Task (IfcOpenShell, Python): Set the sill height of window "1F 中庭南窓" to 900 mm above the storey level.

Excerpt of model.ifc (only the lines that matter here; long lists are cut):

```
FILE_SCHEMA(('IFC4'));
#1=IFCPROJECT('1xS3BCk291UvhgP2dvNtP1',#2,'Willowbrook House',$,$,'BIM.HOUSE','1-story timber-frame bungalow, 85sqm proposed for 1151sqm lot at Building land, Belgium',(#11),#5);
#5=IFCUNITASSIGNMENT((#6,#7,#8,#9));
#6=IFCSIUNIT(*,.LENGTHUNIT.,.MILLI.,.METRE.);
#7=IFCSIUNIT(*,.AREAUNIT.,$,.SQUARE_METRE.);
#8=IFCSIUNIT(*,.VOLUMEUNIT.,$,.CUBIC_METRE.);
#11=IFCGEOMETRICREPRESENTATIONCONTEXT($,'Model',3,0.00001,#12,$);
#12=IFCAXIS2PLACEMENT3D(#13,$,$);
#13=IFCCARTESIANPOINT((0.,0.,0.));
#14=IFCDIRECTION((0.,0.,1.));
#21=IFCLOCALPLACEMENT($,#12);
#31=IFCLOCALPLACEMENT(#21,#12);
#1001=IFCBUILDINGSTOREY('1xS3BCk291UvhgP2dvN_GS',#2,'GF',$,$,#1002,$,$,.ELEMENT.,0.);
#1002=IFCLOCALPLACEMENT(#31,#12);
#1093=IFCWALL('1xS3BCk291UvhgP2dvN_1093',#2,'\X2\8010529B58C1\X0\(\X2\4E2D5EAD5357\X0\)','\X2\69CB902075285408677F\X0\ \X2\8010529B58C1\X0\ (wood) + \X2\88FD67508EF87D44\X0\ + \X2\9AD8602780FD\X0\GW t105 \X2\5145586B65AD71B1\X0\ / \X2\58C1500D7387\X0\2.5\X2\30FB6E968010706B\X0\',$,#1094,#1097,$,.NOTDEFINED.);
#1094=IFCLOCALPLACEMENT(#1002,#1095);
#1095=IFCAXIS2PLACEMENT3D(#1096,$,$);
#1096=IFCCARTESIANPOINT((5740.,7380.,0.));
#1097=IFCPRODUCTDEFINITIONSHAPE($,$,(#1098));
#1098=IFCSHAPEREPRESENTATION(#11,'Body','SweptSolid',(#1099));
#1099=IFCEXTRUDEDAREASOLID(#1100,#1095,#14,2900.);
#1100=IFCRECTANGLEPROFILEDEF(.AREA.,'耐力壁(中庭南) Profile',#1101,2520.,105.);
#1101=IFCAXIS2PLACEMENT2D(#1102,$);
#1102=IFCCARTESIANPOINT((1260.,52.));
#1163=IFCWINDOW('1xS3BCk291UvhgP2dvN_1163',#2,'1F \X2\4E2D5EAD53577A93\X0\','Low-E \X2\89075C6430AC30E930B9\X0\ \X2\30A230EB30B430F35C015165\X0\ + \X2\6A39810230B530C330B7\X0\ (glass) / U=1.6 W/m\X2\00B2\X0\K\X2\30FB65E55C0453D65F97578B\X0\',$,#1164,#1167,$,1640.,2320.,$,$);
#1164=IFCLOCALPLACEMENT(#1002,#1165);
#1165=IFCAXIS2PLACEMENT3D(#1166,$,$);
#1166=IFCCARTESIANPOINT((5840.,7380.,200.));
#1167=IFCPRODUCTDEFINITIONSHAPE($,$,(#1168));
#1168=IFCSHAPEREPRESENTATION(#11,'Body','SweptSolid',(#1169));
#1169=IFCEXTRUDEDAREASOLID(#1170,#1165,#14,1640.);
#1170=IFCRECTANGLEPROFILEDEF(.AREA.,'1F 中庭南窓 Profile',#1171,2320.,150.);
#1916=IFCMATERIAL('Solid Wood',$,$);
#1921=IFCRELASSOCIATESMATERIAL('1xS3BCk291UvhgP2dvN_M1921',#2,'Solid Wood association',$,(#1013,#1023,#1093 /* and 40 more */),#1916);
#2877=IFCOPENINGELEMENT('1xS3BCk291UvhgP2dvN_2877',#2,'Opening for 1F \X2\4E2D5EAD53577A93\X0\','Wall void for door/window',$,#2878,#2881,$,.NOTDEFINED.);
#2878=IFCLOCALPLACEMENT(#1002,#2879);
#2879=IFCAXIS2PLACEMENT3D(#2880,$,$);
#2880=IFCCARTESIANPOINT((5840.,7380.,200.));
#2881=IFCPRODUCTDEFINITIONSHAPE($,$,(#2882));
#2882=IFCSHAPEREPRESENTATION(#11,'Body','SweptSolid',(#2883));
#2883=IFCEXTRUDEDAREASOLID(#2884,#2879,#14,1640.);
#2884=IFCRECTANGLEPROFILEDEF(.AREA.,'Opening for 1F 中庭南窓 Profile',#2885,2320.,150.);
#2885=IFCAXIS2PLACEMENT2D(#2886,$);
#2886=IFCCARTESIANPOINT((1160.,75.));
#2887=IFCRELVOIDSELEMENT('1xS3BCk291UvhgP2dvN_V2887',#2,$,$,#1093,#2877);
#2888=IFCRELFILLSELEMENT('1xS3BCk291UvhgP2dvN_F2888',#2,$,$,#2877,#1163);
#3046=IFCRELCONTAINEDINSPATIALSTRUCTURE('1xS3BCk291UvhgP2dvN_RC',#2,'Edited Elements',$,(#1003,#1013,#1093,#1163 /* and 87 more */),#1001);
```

```python
import numpy as np
import ifcopenshell
import ifcopenshell.api.geometry
import ifcopenshell.geom
import ifcopenshell.util.element
import ifcopenshell.util.placement
import ifcopenshell.util.shape
import ifcopenshell.util.unit

model = ifcopenshell.open("model.ifc")
unit_scale = ifcopenshell.util.unit.calculate_unit_scale(model)

window = model.by_guid("1xS3BCk291UvhgP2dvN_1163")
opening = window.FillsVoids[0].RelatingOpeningElement
storey = ifcopenshell.util.element.get_container(window, ifc_class="IfcBuildingStorey")
level = ifcopenshell.util.placement.get_local_placement(storey.ObjectPlacement)[2, 3]

# The opening's origin need not be at the sill, so measure its lowest point.
shape = ifcopenshell.geom.create_shape(ifcopenshell.geom.settings(), opening)
bottom = ifcopenshell.util.shape.get_shape_bottom_elevation(shape, shape.geometry) / unit_scale
dz = level + 900.0 - bottom

shift = np.array([0.0, 0.0, dz])
# The window is not placed relative to its opening, so move both.
for product in (opening, window):
    matrix = ifcopenshell.util.placement.get_local_placement(product.ObjectPlacement)
    matrix[:3, 3] += shift
    ifcopenshell.api.geometry.edit_object_placement(model, product=product, matrix=matrix, is_si=False)

print(f"moved by {dz * unit_scale:+.3f} m")

model.write("model_updated.ifc")
```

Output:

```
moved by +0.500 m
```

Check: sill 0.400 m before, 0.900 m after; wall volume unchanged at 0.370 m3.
